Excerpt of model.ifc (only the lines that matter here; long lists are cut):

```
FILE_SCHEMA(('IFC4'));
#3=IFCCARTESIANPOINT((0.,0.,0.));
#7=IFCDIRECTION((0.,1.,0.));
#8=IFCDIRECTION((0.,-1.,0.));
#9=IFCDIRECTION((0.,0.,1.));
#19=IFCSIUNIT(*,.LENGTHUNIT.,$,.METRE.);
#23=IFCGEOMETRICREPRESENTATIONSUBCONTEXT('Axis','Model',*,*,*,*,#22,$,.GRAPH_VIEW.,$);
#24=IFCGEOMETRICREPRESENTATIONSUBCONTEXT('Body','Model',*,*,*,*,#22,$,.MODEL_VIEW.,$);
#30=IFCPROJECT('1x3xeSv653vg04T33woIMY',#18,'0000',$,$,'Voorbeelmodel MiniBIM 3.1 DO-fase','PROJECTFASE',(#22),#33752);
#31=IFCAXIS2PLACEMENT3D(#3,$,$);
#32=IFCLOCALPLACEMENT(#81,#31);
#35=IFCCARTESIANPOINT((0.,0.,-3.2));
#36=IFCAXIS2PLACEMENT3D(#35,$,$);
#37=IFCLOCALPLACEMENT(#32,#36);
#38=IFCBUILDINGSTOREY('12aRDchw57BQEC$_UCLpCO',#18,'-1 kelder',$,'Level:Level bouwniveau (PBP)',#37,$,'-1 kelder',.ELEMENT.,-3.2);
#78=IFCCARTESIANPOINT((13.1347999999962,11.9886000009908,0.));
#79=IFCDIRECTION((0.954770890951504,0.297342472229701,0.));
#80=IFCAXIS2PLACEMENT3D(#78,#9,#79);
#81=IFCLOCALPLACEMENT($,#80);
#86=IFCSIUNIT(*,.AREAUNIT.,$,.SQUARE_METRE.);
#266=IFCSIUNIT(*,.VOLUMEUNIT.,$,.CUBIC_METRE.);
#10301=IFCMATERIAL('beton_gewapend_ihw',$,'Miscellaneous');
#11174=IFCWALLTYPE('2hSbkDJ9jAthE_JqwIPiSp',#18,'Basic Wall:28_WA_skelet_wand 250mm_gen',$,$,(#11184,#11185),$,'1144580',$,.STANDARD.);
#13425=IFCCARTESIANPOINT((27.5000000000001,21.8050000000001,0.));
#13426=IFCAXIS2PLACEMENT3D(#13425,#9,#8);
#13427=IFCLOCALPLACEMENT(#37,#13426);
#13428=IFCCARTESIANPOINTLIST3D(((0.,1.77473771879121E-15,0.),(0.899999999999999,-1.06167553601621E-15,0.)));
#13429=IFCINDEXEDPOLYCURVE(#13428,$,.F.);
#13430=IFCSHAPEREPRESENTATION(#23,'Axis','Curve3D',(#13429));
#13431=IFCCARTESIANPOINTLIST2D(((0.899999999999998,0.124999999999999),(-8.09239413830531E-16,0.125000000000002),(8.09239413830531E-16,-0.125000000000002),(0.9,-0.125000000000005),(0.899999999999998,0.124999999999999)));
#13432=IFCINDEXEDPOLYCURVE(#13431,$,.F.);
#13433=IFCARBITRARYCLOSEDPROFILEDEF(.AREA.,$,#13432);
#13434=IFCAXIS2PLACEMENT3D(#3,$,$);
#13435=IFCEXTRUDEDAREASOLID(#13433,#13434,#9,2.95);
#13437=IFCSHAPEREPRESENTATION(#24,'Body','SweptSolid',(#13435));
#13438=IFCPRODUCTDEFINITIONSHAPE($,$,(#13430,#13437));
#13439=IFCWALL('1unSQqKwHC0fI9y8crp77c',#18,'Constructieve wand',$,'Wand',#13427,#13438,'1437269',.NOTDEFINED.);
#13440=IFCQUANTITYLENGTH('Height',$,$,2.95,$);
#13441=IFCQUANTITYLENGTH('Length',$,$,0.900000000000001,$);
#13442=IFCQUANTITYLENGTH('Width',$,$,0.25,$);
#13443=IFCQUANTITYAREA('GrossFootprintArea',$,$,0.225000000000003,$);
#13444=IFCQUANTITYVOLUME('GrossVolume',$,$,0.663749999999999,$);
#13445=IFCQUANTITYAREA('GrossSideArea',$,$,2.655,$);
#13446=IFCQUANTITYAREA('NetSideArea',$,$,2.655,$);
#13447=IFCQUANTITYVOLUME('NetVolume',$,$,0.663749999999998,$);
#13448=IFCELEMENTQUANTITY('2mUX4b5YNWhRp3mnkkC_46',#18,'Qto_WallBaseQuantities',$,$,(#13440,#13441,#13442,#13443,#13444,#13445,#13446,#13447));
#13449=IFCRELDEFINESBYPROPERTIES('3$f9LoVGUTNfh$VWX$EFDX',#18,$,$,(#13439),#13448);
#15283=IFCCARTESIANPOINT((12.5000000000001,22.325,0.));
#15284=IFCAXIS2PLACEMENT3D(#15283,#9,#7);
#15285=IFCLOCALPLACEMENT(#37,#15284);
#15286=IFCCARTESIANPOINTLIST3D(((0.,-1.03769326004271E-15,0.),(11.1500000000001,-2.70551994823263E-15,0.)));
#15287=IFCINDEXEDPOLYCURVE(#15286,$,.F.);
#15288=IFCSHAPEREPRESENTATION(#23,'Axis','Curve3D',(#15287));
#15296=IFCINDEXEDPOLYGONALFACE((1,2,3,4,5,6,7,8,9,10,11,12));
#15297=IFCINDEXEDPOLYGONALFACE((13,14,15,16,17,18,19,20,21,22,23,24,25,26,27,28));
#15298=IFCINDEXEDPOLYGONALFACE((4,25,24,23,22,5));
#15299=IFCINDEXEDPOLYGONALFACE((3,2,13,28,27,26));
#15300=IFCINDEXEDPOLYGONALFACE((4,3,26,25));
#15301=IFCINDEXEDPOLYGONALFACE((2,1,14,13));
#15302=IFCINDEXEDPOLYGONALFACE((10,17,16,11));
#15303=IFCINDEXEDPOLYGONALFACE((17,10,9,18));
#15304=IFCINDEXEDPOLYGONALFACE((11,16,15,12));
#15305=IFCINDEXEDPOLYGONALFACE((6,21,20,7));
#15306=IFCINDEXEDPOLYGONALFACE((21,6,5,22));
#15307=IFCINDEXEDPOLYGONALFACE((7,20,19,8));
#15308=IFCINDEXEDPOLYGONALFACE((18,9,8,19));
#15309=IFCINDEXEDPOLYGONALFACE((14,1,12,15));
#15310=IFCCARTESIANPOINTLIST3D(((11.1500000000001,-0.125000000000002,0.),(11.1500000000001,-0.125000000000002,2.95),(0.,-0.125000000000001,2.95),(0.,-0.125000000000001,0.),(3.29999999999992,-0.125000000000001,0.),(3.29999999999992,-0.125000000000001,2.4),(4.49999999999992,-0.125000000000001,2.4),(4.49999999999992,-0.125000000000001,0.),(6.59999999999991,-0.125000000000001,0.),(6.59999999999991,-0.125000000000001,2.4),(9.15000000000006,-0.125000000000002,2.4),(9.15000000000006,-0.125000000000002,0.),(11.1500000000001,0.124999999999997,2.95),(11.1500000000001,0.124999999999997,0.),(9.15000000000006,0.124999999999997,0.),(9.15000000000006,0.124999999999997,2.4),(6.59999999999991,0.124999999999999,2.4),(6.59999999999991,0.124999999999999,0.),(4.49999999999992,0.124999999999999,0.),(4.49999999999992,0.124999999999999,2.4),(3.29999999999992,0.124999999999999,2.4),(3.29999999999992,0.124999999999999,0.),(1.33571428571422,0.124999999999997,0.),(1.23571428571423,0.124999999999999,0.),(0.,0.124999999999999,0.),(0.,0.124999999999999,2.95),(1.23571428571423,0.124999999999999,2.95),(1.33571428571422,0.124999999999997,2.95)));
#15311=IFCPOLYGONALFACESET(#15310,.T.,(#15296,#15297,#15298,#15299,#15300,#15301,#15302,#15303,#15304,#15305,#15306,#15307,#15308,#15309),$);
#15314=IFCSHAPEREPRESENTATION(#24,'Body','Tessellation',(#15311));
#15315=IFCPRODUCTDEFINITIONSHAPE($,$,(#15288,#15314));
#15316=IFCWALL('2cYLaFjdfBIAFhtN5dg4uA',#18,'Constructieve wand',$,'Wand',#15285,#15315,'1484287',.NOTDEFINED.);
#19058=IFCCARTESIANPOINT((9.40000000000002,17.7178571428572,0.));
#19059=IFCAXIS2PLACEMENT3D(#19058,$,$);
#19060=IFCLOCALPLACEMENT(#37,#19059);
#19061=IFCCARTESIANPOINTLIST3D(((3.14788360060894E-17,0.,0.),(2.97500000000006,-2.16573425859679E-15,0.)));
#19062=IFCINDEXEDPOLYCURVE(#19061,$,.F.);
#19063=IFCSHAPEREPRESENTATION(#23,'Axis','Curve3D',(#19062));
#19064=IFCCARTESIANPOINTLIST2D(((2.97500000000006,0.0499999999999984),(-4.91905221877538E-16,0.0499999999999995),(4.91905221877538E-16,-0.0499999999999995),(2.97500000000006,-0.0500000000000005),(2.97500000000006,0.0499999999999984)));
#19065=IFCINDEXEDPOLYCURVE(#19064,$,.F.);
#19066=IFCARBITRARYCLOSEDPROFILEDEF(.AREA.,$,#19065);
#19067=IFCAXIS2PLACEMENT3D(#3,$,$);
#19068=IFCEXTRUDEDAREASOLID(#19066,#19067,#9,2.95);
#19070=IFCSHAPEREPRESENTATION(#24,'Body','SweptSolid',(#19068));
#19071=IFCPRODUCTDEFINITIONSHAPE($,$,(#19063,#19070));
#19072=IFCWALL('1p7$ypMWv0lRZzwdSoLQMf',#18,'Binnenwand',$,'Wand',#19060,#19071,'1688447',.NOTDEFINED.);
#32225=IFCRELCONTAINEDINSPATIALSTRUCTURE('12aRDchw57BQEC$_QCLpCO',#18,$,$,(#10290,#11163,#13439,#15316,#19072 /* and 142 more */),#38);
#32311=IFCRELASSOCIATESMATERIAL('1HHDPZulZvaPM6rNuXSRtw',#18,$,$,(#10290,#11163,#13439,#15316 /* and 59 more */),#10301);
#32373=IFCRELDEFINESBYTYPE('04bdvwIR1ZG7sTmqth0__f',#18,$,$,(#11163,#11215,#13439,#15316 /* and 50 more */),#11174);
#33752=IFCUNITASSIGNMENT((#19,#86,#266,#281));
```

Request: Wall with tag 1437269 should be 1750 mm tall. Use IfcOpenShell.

```python
import ifcopenshell
import ifcopenshell.api.pset
import ifcopenshell.geom
import ifcopenshell.util.element
import ifcopenshell.util.representation
import ifcopenshell.util.shape
import ifcopenshell.util.unit

model = ifcopenshell.open("model.ifc")
unit_scale = ifcopenshell.util.unit.calculate_unit_scale(model)
area_scale = ifcopenshell.util.unit.calculate_unit_scale(model, "AREAUNIT")
volume_scale = ifcopenshell.util.unit.calculate_unit_scale(model, "VOLUMEUNIT")
settings = ifcopenshell.geom.settings()


def volume(element):
    """Net volume in cubic metres, openings subtracted."""
    shape = ifcopenshell.geom.create_shape(settings, element)
    return ifcopenshell.util.shape.get_volume(shape.geometry)


wall = model.by_guid("1unSQqKwHC0fI9y8crp77c")
before = volume(wall)

body = ifcopenshell.util.representation.get_representation(wall, "Model", "Body")
solid = body.Items[0]
old_height = solid.Depth
solid.Depth = 1.75 / unit_scale
after = volume(wall)
thickness = 0.25  # wall thickness in metres

# Update the stored height, areas and volumes.
qto = model.by_id(ifcopenshell.util.element.get_pset(wall, "Qto_WallBaseQuantities", should_inherit=False)["id"])
ifcopenshell.api.pset.edit_qto(model, qto=qto, properties={
    "Height": solid.Depth,
    "GrossVolume": ifcopenshell.util.element.get_pset(wall, "Qto_WallBaseQuantities", "GrossVolume") * solid.Depth / old_height,
    "GrossSideArea": ifcopenshell.util.element.get_pset(wall, "Qto_WallBaseQuantities", "GrossSideArea") * solid.Depth / old_height,
    "NetSideArea": after / thickness / area_scale,
    "NetVolume": after / volume_scale,
})

print(f"height {old_height:g} -> {solid.Depth:g}, volume {before:.3f} -> {after:.3f} m3")

model.write("model_updated.ifc")
```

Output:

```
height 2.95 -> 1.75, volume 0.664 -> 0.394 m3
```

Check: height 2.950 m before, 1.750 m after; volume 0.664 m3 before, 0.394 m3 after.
